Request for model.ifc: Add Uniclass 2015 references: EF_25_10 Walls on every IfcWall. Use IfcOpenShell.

First a look at what the model holds.

```python
import ifcopenshell

model = ifcopenshell.open("model.ifc")
print(model.schema)
print("classifications:", [c.Name for c in model.by_type("IfcClassification")])
for ifc_class in ("IfcDoor", "IfcRoof", "IfcStair", "IfcWall", "IfcWindow"):
    print(ifc_class, len(model.by_type(ifc_class)))
```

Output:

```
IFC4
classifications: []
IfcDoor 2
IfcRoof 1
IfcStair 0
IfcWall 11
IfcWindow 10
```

```python
import ifcopenshell
import ifcopenshell.api.classification

model = ifcopenshell.open("model.ifc")

system = ifcopenshell.api.classification.add_classification(model, classification="Uniclass 2015")

codes = {
    "IfcWall": ("EF_25_10", "Walls"),
}
for ifc_class, (code, name) in codes.items():
    products = model.by_type(ifc_class)
    ifcopenshell.api.classification.add_reference(
        model, products=products, classification=system, identification=code, name=name
    )
    print(code, len(products))

model.write("model_rev.ifc")
```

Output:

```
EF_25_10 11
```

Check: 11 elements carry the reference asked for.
